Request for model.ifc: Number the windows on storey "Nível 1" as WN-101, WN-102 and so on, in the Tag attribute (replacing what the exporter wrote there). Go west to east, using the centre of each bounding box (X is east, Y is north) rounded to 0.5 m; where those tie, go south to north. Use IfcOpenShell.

First a look at what the model holds.

```python
import ifcopenshell
import ifcopenshell.util.element
import ifcopenshell.util.placement

model = ifcopenshell.open("model.ifc")
print(model.schema)
storey = next(s for s in model.by_type("IfcBuildingStorey") if s.Name == "Nível 1")
windows = [e for e in ifcopenshell.util.element.get_decomposition(storey) if e.is_a("IfcWindow")]
for e in sorted(windows, key=lambda e: e.id()):
    origin = ifcopenshell.util.placement.get_local_placement(e.ObjectPlacement)[:3, 3]
    print(e.id(), e.Tag, e.Name, origin.round(2) + 0.0, sep=" | ")
```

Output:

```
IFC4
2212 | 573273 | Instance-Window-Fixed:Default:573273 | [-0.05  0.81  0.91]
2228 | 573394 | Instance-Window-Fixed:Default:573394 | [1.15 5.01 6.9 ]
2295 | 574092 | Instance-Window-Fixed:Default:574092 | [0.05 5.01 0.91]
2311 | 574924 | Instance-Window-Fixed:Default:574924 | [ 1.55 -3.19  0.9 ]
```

```python
import ifcopenshell
import ifcopenshell.geom
import ifcopenshell.util.element
import ifcopenshell.util.shape

model = ifcopenshell.open("model.ifc")
settings = ifcopenshell.geom.settings()
settings.set("use-world-coords", True)


def centre(element):
    shape = ifcopenshell.geom.create_shape(settings, element)
    return ifcopenshell.util.shape.get_bbox_centroid(shape.geometry)


storey = next(s for s in model.by_type("IfcBuildingStorey") if s.Name == "Nível 1")
windows = [e for e in ifcopenshell.util.element.get_decomposition(storey) if e.is_a("IfcWindow")]

# Insertion points can sit at a corner or the storey origin, so sort by the geometry (in metres).
centres = {e: centre(e) for e in windows}
windows.sort(key=lambda e: (round(centres[e][0] / 0.5), centres[e][1]))

for i, e in enumerate(windows, start=1):
    number = f"WN-1{i:02d}"
    e.Tag = number
    print(e.id(), number)

model.write("model_edited.ifc")
```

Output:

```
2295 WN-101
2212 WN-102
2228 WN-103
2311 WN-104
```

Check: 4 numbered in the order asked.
